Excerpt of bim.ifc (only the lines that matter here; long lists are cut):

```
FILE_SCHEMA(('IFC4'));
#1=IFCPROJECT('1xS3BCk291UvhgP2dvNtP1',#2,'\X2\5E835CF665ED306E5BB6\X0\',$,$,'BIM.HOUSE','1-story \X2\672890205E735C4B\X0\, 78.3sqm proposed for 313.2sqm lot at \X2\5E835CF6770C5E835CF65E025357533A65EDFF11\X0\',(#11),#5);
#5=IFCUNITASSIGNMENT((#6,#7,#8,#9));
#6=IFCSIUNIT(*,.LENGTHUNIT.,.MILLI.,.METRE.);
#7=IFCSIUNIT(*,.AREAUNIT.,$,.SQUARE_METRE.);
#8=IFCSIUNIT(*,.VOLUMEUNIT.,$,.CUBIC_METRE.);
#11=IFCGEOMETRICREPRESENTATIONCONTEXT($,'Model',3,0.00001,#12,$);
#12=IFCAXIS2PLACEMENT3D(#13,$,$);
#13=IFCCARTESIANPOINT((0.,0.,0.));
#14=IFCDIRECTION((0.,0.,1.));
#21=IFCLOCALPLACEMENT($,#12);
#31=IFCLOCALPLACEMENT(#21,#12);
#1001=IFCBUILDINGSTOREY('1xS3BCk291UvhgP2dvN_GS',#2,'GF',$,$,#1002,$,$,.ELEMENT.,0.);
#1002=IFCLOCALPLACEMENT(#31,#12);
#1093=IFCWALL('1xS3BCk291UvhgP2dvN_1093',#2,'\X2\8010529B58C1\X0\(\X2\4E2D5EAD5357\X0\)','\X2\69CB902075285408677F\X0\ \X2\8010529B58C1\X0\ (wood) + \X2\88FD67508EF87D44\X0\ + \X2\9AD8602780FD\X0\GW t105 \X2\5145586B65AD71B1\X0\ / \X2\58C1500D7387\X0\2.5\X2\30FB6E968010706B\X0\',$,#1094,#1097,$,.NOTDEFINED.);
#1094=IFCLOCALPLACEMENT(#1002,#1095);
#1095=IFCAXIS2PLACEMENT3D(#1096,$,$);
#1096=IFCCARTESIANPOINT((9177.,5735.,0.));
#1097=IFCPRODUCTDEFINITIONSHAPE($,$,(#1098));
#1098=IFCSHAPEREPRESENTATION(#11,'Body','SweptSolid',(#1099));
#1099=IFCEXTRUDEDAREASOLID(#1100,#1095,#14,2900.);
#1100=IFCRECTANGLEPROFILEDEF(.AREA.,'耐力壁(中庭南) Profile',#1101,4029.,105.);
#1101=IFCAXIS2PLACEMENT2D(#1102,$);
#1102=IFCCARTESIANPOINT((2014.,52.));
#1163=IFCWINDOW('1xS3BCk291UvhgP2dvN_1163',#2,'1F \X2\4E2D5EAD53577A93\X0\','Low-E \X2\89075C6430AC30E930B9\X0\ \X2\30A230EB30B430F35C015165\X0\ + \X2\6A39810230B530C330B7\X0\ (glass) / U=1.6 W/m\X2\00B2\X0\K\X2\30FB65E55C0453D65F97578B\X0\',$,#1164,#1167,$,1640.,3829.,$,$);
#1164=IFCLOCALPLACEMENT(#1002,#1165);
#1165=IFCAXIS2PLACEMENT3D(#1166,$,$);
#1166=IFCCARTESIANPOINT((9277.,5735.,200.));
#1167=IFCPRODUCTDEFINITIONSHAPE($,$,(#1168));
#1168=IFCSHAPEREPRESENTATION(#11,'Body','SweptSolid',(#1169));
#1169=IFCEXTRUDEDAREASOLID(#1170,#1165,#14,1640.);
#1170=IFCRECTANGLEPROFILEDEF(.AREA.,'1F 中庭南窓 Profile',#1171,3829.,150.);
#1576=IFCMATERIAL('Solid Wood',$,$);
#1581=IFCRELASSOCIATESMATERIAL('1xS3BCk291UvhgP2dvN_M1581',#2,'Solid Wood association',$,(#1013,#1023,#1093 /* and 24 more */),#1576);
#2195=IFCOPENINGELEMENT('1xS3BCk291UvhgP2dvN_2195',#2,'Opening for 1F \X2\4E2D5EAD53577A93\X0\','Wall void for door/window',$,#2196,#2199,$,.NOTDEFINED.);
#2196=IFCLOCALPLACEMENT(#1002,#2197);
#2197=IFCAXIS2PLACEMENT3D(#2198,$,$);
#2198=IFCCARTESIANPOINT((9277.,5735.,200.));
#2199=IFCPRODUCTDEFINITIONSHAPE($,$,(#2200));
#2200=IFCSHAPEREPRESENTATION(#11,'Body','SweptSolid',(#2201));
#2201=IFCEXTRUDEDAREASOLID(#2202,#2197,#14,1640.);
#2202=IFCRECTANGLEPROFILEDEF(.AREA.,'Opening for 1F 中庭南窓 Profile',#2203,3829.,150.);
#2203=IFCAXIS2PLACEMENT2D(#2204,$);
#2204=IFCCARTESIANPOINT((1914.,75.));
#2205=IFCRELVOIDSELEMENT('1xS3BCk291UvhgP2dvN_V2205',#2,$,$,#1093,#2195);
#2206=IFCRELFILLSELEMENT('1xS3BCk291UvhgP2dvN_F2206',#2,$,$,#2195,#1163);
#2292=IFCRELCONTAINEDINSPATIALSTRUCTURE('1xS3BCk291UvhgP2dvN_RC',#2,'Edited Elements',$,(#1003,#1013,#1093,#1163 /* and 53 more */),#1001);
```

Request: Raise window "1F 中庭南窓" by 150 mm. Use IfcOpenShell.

```python
import numpy as np
import ifcopenshell
import ifcopenshell.api.geometry
import ifcopenshell.util.placement
import ifcopenshell.util.unit

model = ifcopenshell.open("bim.ifc")
unit_scale = ifcopenshell.util.unit.calculate_unit_scale(model)

window = model.by_guid("1xS3BCk291UvhgP2dvN_1163")
opening = window.FillsVoids[0].RelatingOpeningElement
dz = 0.15 / unit_scale

shift = np.array([0.0, 0.0, dz])
# The window is not placed relative to its opening, so move both.
for product in (opening, window):
    matrix = ifcopenshell.util.placement.get_local_placement(product.ObjectPlacement)
    matrix[:3, 3] += shift
    ifcopenshell.api.geometry.edit_object_placement(model, product=product, matrix=matrix, is_si=False)

print(f"moved by {dz * unit_scale:+.3f} m")

model.write("bim_rev.ifc")
```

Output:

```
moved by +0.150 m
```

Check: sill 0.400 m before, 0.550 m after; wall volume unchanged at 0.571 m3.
